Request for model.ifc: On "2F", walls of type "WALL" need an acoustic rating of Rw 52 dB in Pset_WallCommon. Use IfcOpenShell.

First a look at what the model holds.

```python
import ifcopenshell
import ifcopenshell.util.element

model = ifcopenshell.open("model.ifc")
print(model.schema)
storey = next(s for s in model.by_type("IfcBuildingStorey") if s.Name == "2F")
walls = [e for e in ifcopenshell.util.element.get_decomposition(storey) if e.is_a("IfcWall")]
seen = {}
for e in walls:
    element_type = ifcopenshell.util.element.get_type(e)
    key = (element_type.Name if element_type != e and element_type else None, ifcopenshell.util.element.get_pset(e, "Pset_WallCommon", "AcousticRating"))
    seen[key] = seen.get(key, 0) + 1
for (name, value), count in sorted(seen.items(), key=str):
    print(count, "x", name, "|", value)
```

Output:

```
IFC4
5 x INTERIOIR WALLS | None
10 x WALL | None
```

```python
import ifcopenshell
import ifcopenshell.api.pset
import ifcopenshell.util.element

model = ifcopenshell.open("model.ifc")

storey = next(s for s in model.by_type("IfcBuildingStorey") if s.Name == "2F")
walls = [e for e in ifcopenshell.util.element.get_decomposition(storey) if e.is_a("IfcWall")]

count = 0
for e in walls:
    element_type = ifcopenshell.util.element.get_type(e)
    if element_type in (None, e) or element_type.Name != "WALL":
        continue
    # add_pset returns the element's existing set when there is one.
    pset = ifcopenshell.api.pset.add_pset(model, product=e, name="Pset_WallCommon")
    ifcopenshell.api.pset.edit_pset(model, pset=pset, properties={"AcousticRating": "Rw 52 dB"})
    count += 1

print(count, "walls updated")

model.write("model_updated.ifc")
```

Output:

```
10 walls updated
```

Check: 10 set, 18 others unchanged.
